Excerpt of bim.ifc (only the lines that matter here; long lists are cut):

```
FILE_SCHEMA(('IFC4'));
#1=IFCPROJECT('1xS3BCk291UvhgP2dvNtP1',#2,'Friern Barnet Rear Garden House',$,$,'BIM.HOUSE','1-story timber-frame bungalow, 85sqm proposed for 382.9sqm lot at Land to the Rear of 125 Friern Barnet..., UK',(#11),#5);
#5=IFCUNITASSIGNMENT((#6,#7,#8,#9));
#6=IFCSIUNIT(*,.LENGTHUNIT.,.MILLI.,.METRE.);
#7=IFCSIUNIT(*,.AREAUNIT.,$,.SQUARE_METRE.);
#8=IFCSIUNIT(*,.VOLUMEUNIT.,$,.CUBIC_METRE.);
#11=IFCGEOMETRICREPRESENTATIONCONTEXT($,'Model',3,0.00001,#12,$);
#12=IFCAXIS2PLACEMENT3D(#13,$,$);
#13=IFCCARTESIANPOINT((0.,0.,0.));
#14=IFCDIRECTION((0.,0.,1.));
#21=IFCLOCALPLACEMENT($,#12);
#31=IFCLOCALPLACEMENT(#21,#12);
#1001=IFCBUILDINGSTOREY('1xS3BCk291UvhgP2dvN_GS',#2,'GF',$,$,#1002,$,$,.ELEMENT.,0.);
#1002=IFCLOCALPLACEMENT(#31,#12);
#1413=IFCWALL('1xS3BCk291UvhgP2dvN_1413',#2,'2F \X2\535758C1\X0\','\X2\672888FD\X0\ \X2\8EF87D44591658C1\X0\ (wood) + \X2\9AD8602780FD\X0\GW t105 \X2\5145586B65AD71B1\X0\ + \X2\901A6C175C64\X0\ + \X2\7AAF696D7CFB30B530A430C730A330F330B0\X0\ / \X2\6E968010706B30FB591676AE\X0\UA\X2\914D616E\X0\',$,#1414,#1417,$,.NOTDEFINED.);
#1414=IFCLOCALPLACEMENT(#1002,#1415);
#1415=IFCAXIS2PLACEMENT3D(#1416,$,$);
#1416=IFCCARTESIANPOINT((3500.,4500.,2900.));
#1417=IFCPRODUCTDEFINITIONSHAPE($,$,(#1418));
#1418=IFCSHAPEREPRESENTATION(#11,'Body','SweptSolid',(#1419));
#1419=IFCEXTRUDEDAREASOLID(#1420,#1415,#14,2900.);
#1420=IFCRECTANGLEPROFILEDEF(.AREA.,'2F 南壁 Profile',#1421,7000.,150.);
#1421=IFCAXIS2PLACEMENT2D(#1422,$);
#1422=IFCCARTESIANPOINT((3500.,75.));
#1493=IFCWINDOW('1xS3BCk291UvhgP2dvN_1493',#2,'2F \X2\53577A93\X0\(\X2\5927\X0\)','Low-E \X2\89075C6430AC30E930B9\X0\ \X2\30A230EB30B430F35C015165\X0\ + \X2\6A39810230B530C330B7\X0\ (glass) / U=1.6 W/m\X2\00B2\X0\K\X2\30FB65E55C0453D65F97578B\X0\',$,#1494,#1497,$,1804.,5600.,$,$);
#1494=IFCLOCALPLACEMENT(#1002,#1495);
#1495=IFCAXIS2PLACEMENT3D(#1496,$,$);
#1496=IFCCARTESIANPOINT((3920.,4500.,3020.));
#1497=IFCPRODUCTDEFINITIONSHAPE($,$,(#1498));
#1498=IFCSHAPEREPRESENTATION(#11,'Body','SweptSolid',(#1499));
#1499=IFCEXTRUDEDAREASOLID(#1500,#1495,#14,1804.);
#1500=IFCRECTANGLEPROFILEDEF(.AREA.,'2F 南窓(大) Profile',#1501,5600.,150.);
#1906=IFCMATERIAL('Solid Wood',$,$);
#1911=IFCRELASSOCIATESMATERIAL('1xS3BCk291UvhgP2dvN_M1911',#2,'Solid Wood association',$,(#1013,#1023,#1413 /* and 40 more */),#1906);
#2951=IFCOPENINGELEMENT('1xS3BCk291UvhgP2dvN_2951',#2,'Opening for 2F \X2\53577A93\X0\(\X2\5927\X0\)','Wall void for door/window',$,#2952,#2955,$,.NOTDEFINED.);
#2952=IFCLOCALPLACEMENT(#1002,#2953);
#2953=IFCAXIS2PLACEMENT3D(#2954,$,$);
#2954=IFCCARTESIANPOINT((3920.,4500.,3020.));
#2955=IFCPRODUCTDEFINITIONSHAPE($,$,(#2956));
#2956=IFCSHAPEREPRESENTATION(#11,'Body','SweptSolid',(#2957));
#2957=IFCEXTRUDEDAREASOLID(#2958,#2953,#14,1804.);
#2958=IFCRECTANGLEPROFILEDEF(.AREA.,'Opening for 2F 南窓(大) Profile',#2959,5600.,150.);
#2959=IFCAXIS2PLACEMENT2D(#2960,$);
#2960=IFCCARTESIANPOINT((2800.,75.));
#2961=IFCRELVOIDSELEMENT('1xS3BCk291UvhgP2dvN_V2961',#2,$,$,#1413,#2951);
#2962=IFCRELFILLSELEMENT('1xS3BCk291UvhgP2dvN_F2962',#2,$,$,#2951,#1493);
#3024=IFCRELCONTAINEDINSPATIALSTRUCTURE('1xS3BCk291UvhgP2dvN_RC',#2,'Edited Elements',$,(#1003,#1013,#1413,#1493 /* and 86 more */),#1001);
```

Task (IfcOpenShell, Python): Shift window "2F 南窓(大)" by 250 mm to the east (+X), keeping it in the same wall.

```python
import ifcopenshell
import ifcopenshell.api.geometry
import ifcopenshell.util.placement
import ifcopenshell.util.unit

model = ifcopenshell.open("bim.ifc")
unit_scale = ifcopenshell.util.unit.calculate_unit_scale(model)

window = model.by_id(1493)
opening = window.FillsVoids[0].RelatingOpeningElement
wall = opening.VoidsElements[0].RelatingBuildingElement

wall_matrix = ifcopenshell.util.placement.get_local_placement(wall.ObjectPlacement)
shift = wall_matrix[:3, 0] * 0.25 / unit_scale
before = ifcopenshell.util.placement.get_local_placement(window.ObjectPlacement)[:3, 3].copy()

# The window is not placed relative to its opening, so move both.
for product in (opening, window):
    matrix = ifcopenshell.util.placement.get_local_placement(product.ObjectPlacement)
    matrix[:3, 3] += shift
    ifcopenshell.api.geometry.edit_object_placement(model, product=product, matrix=matrix, is_si=False)

after = ifcopenshell.util.placement.get_local_placement(window.ObjectPlacement)[:3, 3]
print("window moved by", (after - before).round(3) + 0.0)

model.write("bim_edited.ifc")
```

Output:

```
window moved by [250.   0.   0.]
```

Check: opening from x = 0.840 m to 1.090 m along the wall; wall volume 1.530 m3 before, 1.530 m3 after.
